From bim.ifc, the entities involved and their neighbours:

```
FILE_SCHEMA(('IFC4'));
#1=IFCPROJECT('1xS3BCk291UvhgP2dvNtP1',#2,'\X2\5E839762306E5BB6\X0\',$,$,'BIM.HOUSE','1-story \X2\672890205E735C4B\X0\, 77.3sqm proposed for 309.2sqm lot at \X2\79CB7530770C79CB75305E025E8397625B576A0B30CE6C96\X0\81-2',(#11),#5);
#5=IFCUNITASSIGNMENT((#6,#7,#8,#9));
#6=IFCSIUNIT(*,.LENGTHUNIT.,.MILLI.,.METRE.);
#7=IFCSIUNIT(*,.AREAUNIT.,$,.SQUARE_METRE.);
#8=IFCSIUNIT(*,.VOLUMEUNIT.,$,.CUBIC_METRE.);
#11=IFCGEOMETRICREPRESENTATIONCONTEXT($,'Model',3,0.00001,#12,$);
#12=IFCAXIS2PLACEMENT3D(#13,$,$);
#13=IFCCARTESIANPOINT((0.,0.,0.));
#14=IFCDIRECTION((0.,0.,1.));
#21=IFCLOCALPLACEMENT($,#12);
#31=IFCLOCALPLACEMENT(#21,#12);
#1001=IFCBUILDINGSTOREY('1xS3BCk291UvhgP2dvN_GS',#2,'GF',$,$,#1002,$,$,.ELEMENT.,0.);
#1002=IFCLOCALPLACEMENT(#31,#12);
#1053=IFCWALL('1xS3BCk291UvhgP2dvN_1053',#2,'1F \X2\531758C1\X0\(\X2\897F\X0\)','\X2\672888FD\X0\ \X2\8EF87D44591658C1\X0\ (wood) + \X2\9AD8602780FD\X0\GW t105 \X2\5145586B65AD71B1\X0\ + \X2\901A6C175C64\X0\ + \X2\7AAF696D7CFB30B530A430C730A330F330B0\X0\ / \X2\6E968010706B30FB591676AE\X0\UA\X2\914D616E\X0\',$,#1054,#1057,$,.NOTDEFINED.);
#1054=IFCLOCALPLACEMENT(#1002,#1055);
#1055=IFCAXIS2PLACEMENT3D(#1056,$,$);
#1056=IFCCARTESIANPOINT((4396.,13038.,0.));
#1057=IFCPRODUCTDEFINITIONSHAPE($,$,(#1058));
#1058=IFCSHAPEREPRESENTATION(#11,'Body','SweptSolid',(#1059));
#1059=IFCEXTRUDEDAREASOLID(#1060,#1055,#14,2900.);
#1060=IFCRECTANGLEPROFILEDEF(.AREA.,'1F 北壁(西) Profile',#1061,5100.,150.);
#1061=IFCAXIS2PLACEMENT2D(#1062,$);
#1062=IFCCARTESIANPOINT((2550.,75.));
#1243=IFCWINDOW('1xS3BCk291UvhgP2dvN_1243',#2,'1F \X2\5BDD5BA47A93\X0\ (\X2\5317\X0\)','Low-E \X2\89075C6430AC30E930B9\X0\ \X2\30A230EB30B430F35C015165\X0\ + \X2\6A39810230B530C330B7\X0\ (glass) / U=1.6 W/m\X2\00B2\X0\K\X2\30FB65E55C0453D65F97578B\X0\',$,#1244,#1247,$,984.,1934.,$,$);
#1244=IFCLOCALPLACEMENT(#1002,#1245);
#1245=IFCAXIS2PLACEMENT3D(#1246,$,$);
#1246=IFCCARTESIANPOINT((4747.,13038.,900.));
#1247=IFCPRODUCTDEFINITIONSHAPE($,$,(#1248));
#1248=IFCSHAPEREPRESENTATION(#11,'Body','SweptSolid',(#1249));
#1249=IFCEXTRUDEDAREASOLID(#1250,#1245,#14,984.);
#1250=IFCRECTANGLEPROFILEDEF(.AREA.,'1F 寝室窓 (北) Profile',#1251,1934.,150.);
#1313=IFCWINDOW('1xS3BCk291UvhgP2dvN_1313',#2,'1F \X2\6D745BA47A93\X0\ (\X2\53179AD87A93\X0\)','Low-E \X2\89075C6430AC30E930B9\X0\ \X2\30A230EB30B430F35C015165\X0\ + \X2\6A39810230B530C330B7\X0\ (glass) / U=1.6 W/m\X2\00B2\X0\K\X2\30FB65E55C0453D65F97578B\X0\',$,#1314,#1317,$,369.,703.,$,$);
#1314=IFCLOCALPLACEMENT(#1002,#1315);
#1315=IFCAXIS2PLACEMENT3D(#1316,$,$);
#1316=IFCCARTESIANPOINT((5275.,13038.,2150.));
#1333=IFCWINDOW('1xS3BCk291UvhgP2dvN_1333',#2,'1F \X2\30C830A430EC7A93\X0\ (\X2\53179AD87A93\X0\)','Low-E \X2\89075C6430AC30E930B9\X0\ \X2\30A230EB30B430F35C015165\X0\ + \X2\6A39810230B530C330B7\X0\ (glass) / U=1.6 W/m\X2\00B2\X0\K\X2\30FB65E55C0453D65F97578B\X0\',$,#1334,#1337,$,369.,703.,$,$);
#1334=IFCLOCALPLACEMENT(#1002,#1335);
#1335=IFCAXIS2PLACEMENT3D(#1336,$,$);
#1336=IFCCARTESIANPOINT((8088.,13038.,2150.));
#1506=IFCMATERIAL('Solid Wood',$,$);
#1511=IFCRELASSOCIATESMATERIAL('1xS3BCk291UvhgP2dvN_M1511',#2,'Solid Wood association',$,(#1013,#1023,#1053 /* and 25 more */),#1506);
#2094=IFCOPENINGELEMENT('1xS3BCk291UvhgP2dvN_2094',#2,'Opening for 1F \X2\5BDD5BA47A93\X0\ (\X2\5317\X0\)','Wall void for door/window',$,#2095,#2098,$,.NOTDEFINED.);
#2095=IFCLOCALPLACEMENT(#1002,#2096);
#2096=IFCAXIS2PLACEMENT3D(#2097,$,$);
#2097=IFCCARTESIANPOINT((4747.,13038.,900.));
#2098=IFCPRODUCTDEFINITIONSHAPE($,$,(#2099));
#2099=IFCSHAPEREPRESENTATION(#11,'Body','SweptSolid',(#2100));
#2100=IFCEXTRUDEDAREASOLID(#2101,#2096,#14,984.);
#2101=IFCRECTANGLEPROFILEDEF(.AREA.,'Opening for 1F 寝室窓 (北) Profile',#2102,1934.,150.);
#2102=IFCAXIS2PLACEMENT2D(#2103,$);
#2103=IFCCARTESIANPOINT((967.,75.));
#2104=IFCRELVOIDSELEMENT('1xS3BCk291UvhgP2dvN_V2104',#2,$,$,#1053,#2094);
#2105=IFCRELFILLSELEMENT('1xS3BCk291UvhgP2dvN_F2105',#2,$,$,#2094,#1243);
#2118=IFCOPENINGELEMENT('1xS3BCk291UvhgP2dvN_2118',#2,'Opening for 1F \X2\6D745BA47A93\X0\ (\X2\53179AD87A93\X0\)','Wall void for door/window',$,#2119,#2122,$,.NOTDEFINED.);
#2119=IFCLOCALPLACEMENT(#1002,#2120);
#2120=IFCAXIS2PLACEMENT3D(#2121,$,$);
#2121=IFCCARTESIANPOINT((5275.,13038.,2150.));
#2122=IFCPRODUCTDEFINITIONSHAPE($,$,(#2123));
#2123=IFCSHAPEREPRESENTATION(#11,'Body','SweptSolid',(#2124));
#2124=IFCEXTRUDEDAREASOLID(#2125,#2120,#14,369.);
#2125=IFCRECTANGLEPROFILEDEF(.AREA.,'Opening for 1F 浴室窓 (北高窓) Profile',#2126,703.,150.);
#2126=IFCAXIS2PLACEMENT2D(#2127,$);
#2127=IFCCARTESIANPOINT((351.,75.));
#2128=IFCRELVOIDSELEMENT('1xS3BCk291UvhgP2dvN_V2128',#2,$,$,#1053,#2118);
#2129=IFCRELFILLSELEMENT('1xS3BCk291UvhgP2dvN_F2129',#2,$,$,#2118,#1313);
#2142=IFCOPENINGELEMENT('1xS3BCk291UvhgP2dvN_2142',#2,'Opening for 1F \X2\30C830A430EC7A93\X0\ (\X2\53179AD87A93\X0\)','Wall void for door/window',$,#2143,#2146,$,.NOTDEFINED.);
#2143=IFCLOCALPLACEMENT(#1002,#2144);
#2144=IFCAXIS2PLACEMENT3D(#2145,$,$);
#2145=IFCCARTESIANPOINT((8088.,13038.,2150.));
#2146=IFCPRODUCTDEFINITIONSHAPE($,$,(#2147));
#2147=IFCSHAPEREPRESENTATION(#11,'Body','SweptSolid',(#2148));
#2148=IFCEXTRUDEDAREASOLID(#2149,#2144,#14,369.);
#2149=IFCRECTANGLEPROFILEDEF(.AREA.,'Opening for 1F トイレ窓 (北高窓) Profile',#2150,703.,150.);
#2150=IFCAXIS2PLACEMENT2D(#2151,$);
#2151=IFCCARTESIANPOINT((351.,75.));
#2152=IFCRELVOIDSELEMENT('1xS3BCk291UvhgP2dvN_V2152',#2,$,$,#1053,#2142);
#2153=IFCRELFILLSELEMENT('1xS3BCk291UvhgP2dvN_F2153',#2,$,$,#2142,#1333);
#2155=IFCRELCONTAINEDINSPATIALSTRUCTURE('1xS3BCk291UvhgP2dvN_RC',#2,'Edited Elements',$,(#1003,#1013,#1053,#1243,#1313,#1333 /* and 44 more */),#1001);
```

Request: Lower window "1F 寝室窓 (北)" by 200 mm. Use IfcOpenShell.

```python
import numpy as np
import ifcopenshell
import ifcopenshell.api.geometry
import ifcopenshell.util.placement
import ifcopenshell.util.unit

model = ifcopenshell.open("bim.ifc")
unit_scale = ifcopenshell.util.unit.calculate_unit_scale(model)

window = model.by_id(1243)
opening = window.FillsVoids[0].RelatingOpeningElement
dz = -200.0

shift = np.array([0.0, 0.0, dz])
# The window is not placed relative to its opening, so move both.
for product in (opening, window):
    matrix = ifcopenshell.util.placement.get_local_placement(product.ObjectPlacement)
    matrix[:3, 3] += shift
    ifcopenshell.api.geometry.edit_object_placement(model, product=product, matrix=matrix, is_si=False)

print(f"moved by {dz * unit_scale:+.3f} m")

model.write("bim_rev.ifc")
```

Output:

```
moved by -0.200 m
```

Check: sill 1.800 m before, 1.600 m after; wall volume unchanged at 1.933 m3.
